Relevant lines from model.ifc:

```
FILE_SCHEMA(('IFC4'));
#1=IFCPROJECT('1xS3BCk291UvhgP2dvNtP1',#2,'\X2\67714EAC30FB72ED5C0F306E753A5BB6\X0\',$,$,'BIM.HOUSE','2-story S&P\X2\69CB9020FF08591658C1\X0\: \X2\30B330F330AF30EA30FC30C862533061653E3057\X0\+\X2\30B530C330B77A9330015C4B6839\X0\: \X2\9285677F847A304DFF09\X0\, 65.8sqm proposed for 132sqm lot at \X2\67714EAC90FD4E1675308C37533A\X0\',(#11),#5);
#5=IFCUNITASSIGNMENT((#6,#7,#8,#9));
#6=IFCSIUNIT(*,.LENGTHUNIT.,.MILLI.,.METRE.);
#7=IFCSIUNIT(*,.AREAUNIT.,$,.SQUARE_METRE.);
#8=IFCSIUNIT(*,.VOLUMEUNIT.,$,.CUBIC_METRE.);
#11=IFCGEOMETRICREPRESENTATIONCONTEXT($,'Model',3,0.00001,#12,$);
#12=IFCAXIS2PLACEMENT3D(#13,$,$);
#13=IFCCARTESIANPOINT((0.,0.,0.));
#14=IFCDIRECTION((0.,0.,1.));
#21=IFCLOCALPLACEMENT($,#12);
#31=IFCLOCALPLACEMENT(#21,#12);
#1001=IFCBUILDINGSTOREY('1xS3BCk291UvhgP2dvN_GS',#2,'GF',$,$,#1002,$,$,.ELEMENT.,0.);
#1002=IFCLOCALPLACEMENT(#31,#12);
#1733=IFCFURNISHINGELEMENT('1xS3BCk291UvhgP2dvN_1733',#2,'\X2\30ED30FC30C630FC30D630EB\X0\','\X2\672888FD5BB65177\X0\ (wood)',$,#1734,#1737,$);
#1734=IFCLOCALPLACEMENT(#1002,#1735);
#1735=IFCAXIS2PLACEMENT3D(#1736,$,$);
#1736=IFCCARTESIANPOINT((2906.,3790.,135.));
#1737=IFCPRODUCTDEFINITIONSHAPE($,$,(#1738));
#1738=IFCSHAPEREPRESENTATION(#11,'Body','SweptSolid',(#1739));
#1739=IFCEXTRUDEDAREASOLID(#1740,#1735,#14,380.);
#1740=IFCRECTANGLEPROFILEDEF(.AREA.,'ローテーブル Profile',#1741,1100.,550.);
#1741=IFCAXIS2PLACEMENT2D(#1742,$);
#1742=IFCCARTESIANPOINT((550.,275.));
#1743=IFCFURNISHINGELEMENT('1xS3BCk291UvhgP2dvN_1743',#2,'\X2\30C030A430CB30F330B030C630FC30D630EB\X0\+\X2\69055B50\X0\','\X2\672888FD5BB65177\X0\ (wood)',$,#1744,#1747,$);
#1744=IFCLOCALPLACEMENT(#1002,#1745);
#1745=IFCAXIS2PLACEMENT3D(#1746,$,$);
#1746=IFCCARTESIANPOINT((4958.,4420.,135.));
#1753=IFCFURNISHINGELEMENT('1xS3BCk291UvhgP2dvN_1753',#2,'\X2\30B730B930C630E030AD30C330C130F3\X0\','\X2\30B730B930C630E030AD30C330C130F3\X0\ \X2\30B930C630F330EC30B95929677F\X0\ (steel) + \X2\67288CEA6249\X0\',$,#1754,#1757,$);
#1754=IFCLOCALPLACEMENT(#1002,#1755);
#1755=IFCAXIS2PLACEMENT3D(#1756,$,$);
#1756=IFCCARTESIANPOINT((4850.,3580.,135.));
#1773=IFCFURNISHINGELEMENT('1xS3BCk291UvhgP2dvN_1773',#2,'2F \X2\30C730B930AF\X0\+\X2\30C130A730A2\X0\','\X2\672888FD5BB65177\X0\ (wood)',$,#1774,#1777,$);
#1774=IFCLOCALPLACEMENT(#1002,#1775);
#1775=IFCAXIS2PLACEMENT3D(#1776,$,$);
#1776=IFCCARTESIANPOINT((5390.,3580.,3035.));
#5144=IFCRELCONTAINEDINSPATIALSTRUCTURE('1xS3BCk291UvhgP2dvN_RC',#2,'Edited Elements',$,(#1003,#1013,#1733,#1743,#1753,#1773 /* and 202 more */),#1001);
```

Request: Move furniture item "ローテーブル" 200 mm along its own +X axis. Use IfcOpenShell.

```python
import ifcopenshell
import ifcopenshell.api.geometry
import ifcopenshell.util.placement
import ifcopenshell.util.unit

model = ifcopenshell.open("model.ifc")
unit_scale = ifcopenshell.util.unit.calculate_unit_scale(model)

item = model.by_id(1733)
matrix = ifcopenshell.util.placement.get_local_placement(item.ObjectPlacement)
matrix[:3, 3] += matrix[:3, 0] * 0.2 / unit_scale
ifcopenshell.api.geometry.edit_object_placement(model, product=item, matrix=matrix, is_si=False)

print(ifcopenshell.util.placement.get_local_placement(item.ObjectPlacement).round(3) + 0.0)

model.write("model-out.ifc")
```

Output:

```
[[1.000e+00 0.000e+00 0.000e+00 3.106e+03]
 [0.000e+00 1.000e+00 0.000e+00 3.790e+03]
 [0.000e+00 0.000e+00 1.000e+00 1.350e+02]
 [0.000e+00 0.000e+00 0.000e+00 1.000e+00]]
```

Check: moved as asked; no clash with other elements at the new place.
